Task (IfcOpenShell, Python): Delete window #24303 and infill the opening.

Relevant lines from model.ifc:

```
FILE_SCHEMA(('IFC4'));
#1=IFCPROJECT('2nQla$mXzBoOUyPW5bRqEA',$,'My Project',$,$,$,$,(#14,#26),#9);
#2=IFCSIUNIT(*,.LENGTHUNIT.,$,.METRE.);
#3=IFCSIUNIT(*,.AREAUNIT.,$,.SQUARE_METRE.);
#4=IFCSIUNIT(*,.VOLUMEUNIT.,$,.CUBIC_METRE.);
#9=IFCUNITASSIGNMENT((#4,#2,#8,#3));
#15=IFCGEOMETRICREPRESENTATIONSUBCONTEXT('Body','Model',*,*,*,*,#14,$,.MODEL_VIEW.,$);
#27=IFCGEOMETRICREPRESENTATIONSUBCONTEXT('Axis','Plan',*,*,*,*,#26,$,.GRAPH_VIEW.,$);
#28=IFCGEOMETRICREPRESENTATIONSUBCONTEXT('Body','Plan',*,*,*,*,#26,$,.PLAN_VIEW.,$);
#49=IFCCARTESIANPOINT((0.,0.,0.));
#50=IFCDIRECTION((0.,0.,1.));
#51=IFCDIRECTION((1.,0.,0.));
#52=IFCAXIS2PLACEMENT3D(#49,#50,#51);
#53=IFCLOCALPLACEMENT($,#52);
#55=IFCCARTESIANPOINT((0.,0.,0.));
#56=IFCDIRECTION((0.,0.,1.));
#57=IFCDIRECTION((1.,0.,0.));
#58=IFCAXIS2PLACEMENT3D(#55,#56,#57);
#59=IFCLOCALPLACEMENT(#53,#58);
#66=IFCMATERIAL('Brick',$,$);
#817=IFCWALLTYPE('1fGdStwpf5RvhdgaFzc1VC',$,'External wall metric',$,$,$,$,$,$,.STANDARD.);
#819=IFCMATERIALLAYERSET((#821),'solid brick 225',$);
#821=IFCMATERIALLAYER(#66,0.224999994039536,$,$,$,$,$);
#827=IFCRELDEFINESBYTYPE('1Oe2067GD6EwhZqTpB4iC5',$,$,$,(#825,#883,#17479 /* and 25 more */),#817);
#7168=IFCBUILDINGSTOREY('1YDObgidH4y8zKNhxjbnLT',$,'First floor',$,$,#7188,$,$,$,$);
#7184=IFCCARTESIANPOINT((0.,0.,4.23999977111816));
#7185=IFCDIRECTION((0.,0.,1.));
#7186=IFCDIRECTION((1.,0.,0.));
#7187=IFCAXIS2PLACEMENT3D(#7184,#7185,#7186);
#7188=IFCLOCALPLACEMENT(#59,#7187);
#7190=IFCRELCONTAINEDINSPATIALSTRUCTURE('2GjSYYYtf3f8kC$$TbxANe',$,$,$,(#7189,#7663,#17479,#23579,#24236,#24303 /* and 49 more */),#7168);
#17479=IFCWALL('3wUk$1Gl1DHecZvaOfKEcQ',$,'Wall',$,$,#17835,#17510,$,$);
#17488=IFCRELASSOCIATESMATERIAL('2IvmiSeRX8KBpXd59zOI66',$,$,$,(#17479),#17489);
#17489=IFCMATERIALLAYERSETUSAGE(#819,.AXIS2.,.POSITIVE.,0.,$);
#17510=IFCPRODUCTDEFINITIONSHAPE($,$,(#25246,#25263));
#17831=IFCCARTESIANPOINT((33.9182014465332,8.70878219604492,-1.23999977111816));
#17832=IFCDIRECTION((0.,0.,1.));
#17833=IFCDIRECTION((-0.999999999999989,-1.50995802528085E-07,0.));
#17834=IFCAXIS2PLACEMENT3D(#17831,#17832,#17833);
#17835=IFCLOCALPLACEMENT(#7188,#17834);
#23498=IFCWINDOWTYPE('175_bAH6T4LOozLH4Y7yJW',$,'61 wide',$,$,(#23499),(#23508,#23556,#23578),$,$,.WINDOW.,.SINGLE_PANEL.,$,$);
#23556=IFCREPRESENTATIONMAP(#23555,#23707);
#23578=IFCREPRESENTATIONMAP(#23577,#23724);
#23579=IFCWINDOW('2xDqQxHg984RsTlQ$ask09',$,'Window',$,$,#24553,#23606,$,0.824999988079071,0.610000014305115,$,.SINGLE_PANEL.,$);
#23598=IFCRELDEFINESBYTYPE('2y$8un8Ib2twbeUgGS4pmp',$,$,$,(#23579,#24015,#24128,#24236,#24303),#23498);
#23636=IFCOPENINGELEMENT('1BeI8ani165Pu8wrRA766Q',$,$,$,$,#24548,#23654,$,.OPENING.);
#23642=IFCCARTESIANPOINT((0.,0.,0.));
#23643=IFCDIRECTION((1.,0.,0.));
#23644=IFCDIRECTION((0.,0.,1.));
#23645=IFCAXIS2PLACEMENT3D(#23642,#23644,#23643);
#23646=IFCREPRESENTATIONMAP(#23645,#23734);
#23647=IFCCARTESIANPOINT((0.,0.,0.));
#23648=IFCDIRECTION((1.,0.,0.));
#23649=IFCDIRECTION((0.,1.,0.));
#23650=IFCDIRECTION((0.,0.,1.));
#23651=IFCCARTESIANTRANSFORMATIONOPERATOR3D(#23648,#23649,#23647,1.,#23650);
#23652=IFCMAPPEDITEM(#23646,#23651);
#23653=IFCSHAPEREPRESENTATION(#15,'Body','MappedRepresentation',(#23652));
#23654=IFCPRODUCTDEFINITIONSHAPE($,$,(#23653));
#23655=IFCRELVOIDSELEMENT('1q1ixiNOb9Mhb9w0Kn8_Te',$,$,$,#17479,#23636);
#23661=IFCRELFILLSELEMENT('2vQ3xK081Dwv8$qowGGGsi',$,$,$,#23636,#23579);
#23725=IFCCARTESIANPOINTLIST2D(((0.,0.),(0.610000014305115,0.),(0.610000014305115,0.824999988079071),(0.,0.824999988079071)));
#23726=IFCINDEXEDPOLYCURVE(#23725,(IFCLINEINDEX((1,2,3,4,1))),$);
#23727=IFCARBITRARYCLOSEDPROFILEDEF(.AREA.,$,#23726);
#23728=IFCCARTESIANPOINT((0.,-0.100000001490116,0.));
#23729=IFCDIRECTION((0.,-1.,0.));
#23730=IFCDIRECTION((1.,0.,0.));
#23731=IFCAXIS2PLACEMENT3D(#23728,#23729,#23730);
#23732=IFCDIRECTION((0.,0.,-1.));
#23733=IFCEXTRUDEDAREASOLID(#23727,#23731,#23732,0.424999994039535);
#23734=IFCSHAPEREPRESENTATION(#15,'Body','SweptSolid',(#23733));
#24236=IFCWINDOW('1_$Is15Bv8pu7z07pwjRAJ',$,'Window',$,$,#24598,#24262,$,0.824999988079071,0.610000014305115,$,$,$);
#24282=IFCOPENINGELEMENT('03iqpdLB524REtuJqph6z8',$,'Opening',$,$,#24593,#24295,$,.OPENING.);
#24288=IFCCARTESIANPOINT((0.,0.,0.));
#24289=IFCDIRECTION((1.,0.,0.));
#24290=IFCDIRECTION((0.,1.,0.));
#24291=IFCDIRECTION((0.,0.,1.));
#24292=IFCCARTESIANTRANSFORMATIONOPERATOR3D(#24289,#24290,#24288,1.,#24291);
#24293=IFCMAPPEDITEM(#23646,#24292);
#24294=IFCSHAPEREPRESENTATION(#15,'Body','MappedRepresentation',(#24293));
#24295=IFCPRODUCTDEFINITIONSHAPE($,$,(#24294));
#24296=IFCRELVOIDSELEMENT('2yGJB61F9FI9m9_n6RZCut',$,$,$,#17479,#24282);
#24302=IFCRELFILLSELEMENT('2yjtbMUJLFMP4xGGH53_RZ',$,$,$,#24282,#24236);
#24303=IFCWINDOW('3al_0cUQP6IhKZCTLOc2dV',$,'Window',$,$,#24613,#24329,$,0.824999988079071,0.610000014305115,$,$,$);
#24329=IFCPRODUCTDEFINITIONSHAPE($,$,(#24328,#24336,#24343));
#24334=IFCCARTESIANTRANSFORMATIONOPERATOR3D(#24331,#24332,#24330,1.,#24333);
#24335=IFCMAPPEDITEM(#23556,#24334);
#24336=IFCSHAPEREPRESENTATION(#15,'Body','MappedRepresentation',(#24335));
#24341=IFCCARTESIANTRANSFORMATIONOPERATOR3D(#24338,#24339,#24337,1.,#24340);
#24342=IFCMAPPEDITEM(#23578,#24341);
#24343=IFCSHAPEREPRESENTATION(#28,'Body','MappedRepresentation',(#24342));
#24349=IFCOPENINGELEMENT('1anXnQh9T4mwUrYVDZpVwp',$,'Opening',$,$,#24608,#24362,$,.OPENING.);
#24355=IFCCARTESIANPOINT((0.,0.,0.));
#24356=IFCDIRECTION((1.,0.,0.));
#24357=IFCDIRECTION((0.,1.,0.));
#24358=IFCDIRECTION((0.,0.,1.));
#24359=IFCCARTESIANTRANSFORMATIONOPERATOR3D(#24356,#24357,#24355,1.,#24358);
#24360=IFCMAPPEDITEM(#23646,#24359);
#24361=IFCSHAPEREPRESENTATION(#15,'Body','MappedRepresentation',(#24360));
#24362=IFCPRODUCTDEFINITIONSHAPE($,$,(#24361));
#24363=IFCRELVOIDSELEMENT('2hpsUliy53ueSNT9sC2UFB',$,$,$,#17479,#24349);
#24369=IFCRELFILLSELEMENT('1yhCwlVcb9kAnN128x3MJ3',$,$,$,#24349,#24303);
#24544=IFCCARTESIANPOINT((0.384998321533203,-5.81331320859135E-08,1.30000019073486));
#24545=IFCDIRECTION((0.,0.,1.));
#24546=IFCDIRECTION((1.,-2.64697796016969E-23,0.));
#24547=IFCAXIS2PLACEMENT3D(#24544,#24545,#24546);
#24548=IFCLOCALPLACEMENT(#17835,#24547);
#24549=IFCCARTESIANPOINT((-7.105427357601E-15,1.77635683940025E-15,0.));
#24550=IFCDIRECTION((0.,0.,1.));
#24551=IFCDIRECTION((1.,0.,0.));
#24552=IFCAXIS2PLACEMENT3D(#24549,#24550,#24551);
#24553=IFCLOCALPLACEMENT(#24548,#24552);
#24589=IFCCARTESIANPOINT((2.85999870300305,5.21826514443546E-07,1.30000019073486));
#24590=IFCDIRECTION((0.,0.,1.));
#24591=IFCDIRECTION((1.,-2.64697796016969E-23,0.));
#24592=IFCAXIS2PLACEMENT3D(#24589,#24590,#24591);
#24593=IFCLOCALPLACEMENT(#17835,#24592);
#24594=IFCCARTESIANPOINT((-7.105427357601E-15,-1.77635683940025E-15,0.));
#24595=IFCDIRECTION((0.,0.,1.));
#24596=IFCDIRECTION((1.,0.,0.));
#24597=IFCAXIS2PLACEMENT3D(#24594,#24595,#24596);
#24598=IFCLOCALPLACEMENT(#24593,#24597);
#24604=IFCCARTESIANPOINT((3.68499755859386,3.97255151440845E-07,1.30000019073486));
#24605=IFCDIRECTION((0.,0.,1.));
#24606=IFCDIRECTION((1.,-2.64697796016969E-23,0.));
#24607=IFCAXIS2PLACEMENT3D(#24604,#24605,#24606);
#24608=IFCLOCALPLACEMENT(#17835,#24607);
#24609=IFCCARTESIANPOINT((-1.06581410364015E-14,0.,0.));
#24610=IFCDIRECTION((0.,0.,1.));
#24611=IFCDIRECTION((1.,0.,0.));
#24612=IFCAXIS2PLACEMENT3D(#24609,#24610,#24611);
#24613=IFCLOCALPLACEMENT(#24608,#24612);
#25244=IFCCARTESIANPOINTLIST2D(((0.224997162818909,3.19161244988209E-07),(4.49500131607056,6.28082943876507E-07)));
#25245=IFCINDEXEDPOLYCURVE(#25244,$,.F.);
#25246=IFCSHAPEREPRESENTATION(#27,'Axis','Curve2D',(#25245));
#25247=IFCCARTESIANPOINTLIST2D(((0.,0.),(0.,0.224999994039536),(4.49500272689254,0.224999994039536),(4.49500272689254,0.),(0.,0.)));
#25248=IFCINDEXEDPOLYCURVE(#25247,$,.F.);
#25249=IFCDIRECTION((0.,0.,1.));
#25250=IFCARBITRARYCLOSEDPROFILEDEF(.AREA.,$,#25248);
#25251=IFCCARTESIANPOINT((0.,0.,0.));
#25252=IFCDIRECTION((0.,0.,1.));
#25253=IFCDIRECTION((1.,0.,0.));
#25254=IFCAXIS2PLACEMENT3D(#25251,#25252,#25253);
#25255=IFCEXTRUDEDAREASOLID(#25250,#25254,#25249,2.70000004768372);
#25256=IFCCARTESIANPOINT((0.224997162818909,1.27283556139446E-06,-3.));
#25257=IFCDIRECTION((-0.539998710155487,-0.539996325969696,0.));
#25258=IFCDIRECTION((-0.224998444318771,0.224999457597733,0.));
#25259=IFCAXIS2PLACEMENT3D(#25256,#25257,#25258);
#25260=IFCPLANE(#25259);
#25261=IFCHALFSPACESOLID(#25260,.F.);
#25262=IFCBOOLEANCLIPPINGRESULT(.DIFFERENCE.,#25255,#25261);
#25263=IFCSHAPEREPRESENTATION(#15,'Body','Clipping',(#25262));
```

```python
import ifcopenshell
import ifcopenshell.api.feature
import ifcopenshell.api.root
import ifcopenshell.geom
import ifcopenshell.util.shape

model = ifcopenshell.open("model.ifc")
settings = ifcopenshell.geom.settings()


def volume(element):
    """Net volume in cubic metres, openings subtracted."""
    shape = ifcopenshell.geom.create_shape(settings, element)
    return ifcopenshell.util.shape.get_volume(shape.geometry)


window = model.by_guid("3al_0cUQP6IhKZCTLOc2dV")
opening = window.FillsVoids[0].RelatingOpeningElement
wall = opening.VoidsElements[0].RelatingBuildingElement
before = volume(wall)

ifcopenshell.api.root.remove_product(model, product=window)
ifcopenshell.api.feature.remove_feature(model, feature=opening)

after = volume(wall)

print(f"wall volume {before:.3f} -> {after:.3f} m3")

model.write("model-out.ifc")
```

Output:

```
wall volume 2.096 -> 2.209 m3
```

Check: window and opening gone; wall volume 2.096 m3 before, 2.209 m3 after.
